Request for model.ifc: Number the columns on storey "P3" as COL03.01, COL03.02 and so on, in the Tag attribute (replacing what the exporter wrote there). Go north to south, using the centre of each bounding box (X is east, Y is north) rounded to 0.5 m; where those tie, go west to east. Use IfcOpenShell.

First a look at what the model holds.

```python
import ifcopenshell
import ifcopenshell.util.element
import ifcopenshell.util.placement

model = ifcopenshell.open("model.ifc")
print(model.schema)
storey = next(s for s in model.by_type("IfcBuildingStorey") if s.Name == "P3")
columns = [e for e in ifcopenshell.util.element.get_decomposition(storey) if e.is_a("IfcColumn")]
for e in sorted(columns, key=lambda e: e.id()):
    origin = ifcopenshell.util.placement.get_local_placement(e.ObjectPlacement)[:3, 3]
    print(e.id(), e.Tag, e.Name, origin.round(2) + 0.0, sep=" | ")
```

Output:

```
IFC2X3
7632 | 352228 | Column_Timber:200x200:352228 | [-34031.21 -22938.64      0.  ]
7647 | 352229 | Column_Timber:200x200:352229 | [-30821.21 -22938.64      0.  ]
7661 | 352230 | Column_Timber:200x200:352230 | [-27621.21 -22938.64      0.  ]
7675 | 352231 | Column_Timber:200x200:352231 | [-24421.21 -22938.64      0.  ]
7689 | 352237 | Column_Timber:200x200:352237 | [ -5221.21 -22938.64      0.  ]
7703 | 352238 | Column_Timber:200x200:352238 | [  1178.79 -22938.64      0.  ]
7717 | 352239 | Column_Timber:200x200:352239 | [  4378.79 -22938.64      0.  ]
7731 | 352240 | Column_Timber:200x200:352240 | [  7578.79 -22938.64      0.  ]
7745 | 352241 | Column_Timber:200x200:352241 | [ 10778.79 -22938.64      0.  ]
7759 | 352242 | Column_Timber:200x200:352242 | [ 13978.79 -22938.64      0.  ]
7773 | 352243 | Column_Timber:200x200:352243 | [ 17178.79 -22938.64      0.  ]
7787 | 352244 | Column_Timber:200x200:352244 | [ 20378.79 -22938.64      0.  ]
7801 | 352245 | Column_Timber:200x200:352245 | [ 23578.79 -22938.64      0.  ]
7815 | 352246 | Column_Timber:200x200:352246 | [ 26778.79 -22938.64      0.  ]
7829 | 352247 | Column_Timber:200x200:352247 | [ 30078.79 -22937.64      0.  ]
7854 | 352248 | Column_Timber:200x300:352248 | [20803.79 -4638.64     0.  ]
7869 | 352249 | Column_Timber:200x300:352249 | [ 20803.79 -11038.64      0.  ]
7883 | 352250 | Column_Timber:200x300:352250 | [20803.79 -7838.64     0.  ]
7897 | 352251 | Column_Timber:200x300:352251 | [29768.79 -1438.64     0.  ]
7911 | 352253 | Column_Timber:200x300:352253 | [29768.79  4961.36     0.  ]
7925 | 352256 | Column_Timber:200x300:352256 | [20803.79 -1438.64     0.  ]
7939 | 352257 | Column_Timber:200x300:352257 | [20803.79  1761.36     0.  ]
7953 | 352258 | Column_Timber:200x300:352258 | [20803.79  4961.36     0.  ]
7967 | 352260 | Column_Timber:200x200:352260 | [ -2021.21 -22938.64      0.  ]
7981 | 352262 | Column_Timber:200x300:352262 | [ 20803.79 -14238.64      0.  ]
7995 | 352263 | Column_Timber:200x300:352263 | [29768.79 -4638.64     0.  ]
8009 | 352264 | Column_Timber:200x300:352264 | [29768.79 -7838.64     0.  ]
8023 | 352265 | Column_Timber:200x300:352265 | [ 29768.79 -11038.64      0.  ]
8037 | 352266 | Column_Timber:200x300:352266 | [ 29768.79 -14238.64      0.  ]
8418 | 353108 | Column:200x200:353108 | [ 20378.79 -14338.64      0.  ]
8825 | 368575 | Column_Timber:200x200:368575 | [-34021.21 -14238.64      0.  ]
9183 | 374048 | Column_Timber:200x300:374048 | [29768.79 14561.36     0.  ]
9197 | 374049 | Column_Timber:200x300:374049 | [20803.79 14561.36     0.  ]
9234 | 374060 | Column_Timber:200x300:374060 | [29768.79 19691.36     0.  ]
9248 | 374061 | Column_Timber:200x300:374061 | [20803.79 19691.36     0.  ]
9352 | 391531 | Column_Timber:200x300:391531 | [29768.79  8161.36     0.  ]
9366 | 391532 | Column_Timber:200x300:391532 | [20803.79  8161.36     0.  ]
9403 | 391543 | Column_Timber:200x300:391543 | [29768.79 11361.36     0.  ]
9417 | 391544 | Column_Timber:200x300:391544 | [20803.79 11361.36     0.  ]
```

```python
import ifcopenshell
import ifcopenshell.geom
import ifcopenshell.util.element
import ifcopenshell.util.shape

model = ifcopenshell.open("model.ifc")
settings = ifcopenshell.geom.settings()
settings.set("use-world-coords", True)


def centre(element):
    shape = ifcopenshell.geom.create_shape(settings, element)
    return ifcopenshell.util.shape.get_bbox_centroid(shape.geometry)


storey = next(s for s in model.by_type("IfcBuildingStorey") if s.Name == "P3")
columns = [e for e in ifcopenshell.util.element.get_decomposition(storey) if e.is_a("IfcColumn")]

# Insertion points can sit at a corner or the storey origin, so sort by the geometry (in metres).
centres = {e: centre(e) for e in columns}
columns.sort(key=lambda e: (-round(centres[e][1] / 0.5), centres[e][0]))

for i, e in enumerate(columns, start=1):
    number = f"COL03.{i:02d}"
    e.Tag = number
    print(e.id(), number)

model.write("model_updated.ifc")
```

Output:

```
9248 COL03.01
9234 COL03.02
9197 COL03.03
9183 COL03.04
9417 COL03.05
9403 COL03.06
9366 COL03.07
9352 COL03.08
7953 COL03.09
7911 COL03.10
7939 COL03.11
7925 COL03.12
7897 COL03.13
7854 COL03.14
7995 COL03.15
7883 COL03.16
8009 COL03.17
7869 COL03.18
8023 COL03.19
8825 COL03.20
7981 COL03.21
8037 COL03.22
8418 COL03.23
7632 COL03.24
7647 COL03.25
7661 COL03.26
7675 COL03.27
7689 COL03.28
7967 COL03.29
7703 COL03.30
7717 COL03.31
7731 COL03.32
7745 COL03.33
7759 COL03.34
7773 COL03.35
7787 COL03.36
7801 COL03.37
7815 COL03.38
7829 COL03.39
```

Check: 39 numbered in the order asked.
